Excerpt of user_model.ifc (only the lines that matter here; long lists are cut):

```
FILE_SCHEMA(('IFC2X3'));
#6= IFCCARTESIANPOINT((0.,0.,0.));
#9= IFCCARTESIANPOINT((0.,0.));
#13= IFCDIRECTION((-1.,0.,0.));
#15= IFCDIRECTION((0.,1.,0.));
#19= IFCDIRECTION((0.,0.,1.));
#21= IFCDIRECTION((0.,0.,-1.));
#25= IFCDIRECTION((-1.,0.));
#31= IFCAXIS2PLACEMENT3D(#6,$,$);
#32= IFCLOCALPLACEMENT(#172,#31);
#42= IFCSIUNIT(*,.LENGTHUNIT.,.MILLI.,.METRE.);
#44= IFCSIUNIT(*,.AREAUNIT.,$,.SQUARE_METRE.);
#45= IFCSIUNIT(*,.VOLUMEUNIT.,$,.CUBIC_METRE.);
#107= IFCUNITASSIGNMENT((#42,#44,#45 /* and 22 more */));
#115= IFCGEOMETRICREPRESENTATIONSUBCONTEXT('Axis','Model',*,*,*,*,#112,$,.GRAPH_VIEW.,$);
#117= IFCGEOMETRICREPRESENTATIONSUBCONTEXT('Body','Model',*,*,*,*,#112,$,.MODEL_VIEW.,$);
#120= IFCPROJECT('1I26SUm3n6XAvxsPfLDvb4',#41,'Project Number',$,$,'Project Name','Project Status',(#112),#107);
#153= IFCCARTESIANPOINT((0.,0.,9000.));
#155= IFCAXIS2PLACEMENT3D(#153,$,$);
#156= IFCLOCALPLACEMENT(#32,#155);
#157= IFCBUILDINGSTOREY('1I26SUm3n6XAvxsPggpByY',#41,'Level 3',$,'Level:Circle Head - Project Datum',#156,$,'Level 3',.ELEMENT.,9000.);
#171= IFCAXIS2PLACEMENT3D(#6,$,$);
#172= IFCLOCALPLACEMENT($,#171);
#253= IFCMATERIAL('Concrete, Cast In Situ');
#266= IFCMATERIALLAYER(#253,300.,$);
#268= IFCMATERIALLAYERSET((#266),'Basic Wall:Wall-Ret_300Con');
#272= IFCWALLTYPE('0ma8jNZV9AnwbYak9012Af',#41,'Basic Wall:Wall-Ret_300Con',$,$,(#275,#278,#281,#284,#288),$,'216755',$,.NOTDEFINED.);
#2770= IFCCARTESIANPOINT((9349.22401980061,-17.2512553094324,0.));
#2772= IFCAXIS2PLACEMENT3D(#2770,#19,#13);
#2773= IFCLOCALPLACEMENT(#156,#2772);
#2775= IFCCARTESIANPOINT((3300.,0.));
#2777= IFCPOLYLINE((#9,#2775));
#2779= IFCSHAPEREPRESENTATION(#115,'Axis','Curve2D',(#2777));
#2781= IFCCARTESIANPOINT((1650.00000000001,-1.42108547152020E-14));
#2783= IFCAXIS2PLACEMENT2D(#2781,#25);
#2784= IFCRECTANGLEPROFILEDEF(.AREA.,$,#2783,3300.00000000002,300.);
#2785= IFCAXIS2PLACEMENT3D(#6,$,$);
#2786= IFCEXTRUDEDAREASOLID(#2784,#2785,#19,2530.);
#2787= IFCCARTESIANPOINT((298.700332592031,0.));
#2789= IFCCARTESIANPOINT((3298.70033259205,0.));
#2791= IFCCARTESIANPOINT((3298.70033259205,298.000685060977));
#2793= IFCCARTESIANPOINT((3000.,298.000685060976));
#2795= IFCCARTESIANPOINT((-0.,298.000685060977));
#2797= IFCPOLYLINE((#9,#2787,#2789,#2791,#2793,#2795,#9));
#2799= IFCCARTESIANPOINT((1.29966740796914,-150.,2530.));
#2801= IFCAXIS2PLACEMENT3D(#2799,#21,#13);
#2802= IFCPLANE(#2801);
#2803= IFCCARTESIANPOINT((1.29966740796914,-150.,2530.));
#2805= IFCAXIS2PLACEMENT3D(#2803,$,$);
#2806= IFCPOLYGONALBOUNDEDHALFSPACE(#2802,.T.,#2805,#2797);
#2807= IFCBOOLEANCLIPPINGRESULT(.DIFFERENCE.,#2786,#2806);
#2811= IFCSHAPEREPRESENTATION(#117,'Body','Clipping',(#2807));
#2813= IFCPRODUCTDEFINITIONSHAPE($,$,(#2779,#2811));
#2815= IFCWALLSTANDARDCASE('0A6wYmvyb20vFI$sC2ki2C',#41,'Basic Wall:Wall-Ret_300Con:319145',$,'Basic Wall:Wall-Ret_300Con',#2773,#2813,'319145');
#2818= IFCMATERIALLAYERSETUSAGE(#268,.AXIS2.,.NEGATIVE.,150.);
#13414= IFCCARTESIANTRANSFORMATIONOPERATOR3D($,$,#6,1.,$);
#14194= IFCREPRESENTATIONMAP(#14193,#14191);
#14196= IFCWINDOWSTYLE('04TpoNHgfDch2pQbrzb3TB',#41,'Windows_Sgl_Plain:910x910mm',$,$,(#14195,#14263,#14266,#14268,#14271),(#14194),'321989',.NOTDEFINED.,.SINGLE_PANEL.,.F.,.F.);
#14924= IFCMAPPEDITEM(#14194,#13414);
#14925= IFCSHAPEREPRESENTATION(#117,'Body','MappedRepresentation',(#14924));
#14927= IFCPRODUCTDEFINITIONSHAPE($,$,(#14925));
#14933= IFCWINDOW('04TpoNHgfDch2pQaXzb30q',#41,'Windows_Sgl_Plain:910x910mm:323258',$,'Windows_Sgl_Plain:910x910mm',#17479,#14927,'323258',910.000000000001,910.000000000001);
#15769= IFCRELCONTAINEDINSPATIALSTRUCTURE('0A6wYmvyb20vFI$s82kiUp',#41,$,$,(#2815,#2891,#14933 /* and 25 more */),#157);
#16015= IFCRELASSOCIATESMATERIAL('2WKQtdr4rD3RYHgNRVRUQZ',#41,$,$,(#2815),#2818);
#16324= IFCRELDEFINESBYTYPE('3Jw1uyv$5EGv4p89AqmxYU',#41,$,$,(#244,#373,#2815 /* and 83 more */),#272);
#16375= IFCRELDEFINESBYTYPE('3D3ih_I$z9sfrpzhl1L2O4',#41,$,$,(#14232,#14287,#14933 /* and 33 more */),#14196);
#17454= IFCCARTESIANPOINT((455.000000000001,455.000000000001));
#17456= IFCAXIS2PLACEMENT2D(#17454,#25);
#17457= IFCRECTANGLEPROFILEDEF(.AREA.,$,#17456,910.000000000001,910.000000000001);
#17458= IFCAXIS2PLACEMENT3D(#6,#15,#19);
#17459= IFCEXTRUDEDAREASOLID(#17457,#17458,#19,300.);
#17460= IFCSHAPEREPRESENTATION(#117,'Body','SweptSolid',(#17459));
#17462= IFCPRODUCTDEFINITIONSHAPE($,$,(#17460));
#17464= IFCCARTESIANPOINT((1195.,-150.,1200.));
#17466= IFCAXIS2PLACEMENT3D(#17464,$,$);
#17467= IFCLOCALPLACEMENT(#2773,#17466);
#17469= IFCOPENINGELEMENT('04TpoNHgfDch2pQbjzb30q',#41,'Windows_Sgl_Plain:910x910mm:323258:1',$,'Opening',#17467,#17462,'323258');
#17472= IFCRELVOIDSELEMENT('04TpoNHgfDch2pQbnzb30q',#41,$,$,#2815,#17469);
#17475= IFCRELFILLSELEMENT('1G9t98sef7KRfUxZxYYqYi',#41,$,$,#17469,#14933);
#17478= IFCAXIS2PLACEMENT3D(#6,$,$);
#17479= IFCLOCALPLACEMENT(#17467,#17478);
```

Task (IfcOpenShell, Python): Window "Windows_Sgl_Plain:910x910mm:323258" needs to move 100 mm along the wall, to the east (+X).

```python
import ifcopenshell
import ifcopenshell.api.geometry
import ifcopenshell.util.placement

model = ifcopenshell.open("user_model.ifc")

window = model.by_guid("04TpoNHgfDch2pQaXzb30q")
opening = window.FillsVoids[0].RelatingOpeningElement
wall = opening.VoidsElements[0].RelatingBuildingElement

wall_matrix = ifcopenshell.util.placement.get_local_placement(wall.ObjectPlacement)
shift = wall_matrix[:3, 0] * -100.0
before = ifcopenshell.util.placement.get_local_placement(window.ObjectPlacement)[:3, 3].copy()

# The window is placed relative to its opening, so it follows when the opening moves.
matrix = ifcopenshell.util.placement.get_local_placement(opening.ObjectPlacement)
matrix[:3, 3] += shift
ifcopenshell.api.geometry.edit_object_placement(
    model, product=opening, matrix=matrix, is_si=False, should_transform_children=True
)

after = ifcopenshell.util.placement.get_local_placement(window.ObjectPlacement)[:3, 3]
print("window moved by", (after - before).round(3) + 0.0)

model.write("user_model_rev.ifc")
```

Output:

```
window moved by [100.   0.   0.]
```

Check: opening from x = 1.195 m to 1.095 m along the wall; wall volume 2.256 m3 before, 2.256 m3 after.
